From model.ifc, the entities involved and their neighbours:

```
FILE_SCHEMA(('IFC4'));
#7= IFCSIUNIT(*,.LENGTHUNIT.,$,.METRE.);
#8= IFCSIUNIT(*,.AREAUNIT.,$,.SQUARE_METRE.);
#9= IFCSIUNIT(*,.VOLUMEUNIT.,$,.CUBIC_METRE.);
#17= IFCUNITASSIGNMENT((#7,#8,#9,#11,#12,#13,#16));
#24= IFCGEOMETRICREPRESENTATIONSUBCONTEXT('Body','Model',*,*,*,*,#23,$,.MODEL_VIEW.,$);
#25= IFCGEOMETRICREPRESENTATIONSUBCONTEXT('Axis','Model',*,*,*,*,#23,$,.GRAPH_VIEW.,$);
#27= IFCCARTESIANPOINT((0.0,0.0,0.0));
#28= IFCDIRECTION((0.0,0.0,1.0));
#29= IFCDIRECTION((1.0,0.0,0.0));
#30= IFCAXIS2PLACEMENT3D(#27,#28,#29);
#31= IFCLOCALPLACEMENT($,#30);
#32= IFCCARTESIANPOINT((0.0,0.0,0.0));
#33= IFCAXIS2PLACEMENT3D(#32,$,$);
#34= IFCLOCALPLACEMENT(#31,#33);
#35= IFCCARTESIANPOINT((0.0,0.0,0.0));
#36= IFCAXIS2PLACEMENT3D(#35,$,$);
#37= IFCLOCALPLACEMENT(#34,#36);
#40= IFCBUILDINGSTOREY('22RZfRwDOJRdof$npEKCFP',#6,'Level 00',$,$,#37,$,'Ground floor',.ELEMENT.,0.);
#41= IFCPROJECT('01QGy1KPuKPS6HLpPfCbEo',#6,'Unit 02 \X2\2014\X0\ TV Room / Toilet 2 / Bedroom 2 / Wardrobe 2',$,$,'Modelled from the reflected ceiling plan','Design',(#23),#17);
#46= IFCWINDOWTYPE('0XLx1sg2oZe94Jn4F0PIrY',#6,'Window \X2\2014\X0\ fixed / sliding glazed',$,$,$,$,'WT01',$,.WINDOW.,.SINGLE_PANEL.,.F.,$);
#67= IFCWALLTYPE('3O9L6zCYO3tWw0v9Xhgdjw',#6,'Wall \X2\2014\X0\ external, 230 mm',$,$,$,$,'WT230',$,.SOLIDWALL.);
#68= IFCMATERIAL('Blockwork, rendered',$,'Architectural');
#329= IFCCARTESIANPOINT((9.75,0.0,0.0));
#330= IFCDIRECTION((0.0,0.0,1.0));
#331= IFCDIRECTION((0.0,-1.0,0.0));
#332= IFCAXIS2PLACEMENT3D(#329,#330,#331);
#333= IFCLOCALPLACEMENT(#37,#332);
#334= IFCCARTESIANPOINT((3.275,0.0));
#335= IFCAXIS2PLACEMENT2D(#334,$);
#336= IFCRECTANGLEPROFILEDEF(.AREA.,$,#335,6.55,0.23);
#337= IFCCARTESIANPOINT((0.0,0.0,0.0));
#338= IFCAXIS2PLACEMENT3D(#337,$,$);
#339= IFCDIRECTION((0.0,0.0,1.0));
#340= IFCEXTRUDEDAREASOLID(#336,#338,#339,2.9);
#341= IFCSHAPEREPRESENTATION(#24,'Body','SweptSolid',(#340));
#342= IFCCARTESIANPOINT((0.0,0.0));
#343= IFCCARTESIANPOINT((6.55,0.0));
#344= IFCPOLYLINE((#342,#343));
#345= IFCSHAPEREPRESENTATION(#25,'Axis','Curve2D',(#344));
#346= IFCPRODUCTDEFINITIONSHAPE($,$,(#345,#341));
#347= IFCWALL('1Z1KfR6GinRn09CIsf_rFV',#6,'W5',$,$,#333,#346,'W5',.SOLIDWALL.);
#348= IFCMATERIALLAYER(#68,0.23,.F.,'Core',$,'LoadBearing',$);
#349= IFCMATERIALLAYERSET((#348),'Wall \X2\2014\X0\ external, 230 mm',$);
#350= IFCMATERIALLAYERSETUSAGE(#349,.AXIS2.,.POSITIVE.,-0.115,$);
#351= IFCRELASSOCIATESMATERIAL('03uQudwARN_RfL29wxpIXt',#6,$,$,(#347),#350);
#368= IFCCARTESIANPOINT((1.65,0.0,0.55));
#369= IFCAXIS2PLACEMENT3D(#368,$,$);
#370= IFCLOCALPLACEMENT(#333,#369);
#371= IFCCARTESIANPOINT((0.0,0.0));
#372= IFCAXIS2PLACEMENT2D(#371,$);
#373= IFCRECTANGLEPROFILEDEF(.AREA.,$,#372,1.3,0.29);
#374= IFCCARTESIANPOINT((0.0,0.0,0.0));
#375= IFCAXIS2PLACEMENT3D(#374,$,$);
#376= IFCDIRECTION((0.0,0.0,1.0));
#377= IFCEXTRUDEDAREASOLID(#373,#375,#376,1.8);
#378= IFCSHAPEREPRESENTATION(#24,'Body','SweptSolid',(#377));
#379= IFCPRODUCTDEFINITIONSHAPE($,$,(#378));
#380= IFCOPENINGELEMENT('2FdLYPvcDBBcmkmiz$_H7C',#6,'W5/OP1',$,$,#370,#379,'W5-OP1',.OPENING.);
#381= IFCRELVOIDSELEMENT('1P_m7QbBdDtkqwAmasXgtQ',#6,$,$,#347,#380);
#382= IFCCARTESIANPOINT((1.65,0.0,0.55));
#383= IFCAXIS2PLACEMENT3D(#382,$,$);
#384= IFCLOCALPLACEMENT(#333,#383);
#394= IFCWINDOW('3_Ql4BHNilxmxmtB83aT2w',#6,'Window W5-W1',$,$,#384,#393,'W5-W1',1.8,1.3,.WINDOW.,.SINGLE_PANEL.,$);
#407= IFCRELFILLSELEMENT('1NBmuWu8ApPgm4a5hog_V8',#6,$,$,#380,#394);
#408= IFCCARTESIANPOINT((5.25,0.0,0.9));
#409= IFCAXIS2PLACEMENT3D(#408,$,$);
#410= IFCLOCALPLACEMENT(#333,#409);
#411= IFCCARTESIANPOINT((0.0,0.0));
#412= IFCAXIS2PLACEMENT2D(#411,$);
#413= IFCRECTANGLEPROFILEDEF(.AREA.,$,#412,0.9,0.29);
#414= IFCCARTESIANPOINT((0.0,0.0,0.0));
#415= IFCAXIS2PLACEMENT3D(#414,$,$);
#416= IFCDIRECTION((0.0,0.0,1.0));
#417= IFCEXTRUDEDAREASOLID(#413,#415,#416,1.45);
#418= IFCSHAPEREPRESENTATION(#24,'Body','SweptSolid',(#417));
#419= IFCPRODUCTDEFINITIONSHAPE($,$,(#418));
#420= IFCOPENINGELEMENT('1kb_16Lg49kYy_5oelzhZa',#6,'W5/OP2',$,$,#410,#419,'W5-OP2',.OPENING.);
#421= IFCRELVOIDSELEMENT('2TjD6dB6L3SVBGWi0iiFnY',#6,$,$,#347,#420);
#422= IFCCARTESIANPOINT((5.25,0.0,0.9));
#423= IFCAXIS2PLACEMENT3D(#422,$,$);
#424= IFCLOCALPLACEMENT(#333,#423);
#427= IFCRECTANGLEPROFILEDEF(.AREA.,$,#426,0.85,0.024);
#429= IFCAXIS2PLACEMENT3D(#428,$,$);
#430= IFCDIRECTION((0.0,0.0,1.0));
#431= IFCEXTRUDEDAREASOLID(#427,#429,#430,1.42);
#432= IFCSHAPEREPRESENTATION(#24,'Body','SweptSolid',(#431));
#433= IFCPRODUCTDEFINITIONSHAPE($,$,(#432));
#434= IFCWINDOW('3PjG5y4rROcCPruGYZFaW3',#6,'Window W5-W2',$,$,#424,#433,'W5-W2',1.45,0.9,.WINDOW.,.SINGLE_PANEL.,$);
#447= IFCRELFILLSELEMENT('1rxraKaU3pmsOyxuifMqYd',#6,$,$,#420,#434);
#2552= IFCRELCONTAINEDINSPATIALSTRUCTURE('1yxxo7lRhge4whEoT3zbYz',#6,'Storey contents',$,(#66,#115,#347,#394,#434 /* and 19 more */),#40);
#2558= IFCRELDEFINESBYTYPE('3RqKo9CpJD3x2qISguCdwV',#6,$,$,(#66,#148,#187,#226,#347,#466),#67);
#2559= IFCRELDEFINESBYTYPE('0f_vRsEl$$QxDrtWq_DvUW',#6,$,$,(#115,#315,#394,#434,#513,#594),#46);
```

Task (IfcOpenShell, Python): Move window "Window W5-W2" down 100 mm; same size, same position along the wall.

```python
import numpy as np
import ifcopenshell
import ifcopenshell.api.geometry
import ifcopenshell.util.placement
import ifcopenshell.util.unit

model = ifcopenshell.open("model.ifc")
unit_scale = ifcopenshell.util.unit.calculate_unit_scale(model)

window = model.by_id(434)
opening = window.FillsVoids[0].RelatingOpeningElement
dz = -0.1 / unit_scale

shift = np.array([0.0, 0.0, dz])
# The window is not placed relative to its opening, so move both.
for product in (opening, window):
    matrix = ifcopenshell.util.placement.get_local_placement(product.ObjectPlacement)
    matrix[:3, 3] += shift
    ifcopenshell.api.geometry.edit_object_placement(model, product=product, matrix=matrix, is_si=False)

print(f"moved by {dz * unit_scale:+.3f} m")

model.write("model_edited.ifc")
```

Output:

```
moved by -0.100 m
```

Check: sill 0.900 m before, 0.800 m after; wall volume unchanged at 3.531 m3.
